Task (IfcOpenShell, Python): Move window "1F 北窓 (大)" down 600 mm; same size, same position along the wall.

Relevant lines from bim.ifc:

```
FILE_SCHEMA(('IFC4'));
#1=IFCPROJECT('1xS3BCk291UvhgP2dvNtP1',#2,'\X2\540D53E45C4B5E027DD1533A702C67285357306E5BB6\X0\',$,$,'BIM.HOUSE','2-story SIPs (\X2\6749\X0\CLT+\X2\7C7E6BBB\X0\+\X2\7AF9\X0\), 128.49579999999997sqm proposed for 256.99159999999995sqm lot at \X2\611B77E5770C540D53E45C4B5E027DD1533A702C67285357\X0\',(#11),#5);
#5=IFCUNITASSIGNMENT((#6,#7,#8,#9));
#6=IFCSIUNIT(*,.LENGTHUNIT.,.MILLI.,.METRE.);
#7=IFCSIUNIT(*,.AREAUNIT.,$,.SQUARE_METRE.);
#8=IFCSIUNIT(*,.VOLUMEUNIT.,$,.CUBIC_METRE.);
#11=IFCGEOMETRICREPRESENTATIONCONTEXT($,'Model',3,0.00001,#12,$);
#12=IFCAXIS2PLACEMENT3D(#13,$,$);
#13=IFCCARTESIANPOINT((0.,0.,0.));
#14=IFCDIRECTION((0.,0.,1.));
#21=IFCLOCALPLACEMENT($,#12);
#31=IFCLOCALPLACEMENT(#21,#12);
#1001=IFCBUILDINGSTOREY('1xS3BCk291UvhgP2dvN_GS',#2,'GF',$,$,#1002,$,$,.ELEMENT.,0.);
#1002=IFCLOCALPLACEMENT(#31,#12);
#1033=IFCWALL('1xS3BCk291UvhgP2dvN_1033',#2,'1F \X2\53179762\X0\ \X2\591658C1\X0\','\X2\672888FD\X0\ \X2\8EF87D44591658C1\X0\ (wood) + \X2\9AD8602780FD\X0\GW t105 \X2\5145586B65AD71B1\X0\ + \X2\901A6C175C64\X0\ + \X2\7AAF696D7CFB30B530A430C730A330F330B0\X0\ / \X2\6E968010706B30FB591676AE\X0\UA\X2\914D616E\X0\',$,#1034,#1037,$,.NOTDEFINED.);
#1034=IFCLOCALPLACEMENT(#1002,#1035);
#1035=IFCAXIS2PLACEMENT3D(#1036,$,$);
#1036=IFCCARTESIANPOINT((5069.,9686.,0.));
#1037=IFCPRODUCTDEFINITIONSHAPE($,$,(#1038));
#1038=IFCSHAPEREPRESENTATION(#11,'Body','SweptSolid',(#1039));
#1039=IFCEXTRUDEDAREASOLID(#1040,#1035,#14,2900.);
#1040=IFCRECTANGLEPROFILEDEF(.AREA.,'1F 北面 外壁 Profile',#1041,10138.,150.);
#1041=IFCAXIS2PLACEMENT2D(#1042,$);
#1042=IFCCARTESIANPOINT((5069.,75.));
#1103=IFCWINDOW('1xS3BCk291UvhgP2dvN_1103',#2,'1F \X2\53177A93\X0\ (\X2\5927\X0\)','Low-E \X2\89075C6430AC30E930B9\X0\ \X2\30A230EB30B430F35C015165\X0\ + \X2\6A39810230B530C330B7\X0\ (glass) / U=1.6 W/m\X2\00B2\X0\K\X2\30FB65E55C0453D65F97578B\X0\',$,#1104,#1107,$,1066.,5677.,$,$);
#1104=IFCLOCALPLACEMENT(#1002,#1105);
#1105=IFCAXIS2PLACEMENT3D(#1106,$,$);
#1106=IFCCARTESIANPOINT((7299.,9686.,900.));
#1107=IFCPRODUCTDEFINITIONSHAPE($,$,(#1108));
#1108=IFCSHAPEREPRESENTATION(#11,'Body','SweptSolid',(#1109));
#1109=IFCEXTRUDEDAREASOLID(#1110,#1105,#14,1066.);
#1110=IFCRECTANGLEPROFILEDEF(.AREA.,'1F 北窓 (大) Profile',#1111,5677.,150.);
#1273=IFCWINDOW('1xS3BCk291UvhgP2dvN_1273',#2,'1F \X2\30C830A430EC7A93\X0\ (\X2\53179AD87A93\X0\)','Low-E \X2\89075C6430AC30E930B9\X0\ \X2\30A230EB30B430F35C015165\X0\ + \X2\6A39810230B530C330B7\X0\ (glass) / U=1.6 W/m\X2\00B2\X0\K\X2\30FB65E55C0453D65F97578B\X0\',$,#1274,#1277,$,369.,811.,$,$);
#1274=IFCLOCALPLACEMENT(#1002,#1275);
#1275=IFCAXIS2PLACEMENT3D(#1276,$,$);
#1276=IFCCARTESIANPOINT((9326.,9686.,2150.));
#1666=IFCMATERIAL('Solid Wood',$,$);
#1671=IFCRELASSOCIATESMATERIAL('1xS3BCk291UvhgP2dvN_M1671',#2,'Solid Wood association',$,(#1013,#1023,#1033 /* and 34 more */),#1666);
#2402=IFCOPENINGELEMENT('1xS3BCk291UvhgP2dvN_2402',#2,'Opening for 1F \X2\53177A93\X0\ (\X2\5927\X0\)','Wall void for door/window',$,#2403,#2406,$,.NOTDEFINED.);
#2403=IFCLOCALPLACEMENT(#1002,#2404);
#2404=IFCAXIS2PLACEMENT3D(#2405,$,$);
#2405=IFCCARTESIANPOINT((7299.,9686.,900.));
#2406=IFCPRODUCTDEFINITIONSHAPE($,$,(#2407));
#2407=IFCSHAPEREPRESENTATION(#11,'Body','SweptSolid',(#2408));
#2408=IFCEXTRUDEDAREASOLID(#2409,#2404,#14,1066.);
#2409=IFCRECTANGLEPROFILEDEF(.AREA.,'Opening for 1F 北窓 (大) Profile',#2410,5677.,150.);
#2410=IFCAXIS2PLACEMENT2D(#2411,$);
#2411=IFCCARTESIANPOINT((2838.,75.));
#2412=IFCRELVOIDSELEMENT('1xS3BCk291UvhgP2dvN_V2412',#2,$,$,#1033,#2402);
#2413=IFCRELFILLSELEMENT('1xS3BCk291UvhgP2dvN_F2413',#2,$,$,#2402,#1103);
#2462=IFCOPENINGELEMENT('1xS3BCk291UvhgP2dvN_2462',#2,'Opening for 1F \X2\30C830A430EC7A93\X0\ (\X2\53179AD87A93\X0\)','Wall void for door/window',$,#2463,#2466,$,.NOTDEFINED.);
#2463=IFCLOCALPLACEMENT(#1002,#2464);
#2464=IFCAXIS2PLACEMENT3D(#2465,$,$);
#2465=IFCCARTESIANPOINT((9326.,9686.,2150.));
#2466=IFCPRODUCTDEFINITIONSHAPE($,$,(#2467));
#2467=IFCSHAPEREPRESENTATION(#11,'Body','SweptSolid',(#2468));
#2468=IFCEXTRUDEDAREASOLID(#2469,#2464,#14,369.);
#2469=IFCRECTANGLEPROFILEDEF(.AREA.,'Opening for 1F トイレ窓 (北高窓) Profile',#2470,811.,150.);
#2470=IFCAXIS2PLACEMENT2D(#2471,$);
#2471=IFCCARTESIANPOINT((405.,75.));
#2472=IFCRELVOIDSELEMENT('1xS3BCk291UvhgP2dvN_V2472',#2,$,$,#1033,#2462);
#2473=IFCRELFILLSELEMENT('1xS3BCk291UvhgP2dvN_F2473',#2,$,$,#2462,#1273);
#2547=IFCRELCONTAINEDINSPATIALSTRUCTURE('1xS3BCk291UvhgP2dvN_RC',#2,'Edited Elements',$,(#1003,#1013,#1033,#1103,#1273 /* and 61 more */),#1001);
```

```python
import numpy as np
import ifcopenshell
import ifcopenshell.api.geometry
import ifcopenshell.util.placement
import ifcopenshell.util.unit

model = ifcopenshell.open("bim.ifc")
unit_scale = ifcopenshell.util.unit.calculate_unit_scale(model)

window = model.by_guid("1xS3BCk291UvhgP2dvN_1103")
opening = window.FillsVoids[0].RelatingOpeningElement
dz = -600.0

shift = np.array([0.0, 0.0, dz])
# The window is not placed relative to its opening, so move both.
for product in (opening, window):
    matrix = ifcopenshell.util.placement.get_local_placement(product.ObjectPlacement)
    matrix[:3, 3] += shift
    ifcopenshell.api.geometry.edit_object_placement(model, product=product, matrix=matrix, is_si=False)

print(f"moved by {dz * unit_scale:+.3f} m")

model.write("bim_v2.ifc")
```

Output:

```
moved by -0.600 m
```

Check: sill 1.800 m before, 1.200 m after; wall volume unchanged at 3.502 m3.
